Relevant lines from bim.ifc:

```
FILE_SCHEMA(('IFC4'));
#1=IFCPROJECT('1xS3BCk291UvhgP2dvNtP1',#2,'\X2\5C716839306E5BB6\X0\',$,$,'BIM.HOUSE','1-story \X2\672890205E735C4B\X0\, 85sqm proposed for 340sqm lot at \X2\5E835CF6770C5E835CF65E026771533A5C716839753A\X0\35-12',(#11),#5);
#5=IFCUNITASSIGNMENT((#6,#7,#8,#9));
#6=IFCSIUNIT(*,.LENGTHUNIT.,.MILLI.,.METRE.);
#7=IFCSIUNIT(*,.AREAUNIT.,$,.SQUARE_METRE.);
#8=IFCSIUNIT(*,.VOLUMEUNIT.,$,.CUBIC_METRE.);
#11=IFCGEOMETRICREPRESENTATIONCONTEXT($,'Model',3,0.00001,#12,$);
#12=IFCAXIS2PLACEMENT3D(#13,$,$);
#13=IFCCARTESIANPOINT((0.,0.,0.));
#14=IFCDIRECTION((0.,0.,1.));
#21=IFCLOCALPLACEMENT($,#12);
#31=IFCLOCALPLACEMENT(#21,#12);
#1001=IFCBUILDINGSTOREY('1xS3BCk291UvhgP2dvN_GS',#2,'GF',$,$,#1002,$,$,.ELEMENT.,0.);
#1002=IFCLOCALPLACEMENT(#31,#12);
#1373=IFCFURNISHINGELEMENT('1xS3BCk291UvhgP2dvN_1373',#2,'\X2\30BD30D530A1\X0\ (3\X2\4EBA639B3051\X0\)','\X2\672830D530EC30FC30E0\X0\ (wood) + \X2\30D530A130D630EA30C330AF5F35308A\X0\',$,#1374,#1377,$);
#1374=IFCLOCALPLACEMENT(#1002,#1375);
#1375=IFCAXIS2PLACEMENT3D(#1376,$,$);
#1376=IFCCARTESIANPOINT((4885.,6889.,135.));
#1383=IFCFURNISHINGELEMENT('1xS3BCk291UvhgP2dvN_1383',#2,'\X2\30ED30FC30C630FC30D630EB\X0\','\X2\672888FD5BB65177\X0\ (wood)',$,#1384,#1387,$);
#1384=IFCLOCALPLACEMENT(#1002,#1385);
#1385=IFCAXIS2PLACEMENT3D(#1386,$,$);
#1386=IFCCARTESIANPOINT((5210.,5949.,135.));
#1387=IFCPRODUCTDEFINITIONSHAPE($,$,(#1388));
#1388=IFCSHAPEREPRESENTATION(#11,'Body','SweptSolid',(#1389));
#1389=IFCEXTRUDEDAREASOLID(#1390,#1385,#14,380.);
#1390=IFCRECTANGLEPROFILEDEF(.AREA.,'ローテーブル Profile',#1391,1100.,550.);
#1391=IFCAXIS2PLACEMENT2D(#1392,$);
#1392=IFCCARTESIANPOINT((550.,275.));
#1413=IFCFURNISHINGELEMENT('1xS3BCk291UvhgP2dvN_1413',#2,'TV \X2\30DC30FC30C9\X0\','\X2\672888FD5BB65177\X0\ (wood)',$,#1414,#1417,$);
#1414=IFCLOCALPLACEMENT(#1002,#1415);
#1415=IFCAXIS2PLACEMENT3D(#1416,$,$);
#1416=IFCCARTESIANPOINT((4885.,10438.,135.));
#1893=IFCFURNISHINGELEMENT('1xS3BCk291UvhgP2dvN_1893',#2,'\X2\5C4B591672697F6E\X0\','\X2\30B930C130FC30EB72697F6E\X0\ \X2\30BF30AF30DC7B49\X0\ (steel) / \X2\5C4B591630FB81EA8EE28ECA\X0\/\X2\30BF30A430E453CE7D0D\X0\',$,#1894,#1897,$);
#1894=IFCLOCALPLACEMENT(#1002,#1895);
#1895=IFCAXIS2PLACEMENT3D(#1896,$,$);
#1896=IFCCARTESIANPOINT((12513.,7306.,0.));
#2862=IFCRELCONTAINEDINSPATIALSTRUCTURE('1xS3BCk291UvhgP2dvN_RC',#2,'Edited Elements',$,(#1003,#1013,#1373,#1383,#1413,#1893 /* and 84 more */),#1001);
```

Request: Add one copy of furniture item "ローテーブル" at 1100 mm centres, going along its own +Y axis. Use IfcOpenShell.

```python
import ifcopenshell
import ifcopenshell.api.geometry
import ifcopenshell.api.root
import ifcopenshell.util.element
import ifcopenshell.util.placement
import ifcopenshell.util.unit

model = ifcopenshell.open("bim.ifc")
unit_scale = ifcopenshell.util.unit.calculate_unit_scale(model)


def reuse_history(source, copy):
    """copy_class also copies each property set's owner history, people and application; keep the originals."""
    for rel in copy.IsDefinedBy:
        if rel.is_a("IfcRelDefinesByProperties") and (history := rel.RelatingPropertyDefinition.OwnerHistory):
            rel.RelatingPropertyDefinition.OwnerHistory = source.OwnerHistory
            ifcopenshell.util.element.remove_deep2(model, history)


source = model.by_guid("1xS3BCk291UvhgP2dvN_1383")
base = ifcopenshell.util.placement.get_local_placement(source.ObjectPlacement)
step = base[:3, 1] * 1.1 / unit_scale

for i in range(1, 2):
    copy = ifcopenshell.api.root.copy_class(model, product=source)
    copy.Representation = ifcopenshell.util.element.copy_deep(
        model, source.Representation, exclude=["IfcGeometricRepresentationContext", "IfcRepresentationMap"]
    )
    reuse_history(source, copy)
    matrix = base.copy()
    matrix[:3, 3] += i * step
    print("added at", matrix[:3, 3].round(3) + 0.0)
    ifcopenshell.api.geometry.edit_object_placement(model, product=copy, matrix=matrix, is_si=False)

model.write("bim_v2.ifc")
```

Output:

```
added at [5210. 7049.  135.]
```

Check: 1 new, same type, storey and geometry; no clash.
